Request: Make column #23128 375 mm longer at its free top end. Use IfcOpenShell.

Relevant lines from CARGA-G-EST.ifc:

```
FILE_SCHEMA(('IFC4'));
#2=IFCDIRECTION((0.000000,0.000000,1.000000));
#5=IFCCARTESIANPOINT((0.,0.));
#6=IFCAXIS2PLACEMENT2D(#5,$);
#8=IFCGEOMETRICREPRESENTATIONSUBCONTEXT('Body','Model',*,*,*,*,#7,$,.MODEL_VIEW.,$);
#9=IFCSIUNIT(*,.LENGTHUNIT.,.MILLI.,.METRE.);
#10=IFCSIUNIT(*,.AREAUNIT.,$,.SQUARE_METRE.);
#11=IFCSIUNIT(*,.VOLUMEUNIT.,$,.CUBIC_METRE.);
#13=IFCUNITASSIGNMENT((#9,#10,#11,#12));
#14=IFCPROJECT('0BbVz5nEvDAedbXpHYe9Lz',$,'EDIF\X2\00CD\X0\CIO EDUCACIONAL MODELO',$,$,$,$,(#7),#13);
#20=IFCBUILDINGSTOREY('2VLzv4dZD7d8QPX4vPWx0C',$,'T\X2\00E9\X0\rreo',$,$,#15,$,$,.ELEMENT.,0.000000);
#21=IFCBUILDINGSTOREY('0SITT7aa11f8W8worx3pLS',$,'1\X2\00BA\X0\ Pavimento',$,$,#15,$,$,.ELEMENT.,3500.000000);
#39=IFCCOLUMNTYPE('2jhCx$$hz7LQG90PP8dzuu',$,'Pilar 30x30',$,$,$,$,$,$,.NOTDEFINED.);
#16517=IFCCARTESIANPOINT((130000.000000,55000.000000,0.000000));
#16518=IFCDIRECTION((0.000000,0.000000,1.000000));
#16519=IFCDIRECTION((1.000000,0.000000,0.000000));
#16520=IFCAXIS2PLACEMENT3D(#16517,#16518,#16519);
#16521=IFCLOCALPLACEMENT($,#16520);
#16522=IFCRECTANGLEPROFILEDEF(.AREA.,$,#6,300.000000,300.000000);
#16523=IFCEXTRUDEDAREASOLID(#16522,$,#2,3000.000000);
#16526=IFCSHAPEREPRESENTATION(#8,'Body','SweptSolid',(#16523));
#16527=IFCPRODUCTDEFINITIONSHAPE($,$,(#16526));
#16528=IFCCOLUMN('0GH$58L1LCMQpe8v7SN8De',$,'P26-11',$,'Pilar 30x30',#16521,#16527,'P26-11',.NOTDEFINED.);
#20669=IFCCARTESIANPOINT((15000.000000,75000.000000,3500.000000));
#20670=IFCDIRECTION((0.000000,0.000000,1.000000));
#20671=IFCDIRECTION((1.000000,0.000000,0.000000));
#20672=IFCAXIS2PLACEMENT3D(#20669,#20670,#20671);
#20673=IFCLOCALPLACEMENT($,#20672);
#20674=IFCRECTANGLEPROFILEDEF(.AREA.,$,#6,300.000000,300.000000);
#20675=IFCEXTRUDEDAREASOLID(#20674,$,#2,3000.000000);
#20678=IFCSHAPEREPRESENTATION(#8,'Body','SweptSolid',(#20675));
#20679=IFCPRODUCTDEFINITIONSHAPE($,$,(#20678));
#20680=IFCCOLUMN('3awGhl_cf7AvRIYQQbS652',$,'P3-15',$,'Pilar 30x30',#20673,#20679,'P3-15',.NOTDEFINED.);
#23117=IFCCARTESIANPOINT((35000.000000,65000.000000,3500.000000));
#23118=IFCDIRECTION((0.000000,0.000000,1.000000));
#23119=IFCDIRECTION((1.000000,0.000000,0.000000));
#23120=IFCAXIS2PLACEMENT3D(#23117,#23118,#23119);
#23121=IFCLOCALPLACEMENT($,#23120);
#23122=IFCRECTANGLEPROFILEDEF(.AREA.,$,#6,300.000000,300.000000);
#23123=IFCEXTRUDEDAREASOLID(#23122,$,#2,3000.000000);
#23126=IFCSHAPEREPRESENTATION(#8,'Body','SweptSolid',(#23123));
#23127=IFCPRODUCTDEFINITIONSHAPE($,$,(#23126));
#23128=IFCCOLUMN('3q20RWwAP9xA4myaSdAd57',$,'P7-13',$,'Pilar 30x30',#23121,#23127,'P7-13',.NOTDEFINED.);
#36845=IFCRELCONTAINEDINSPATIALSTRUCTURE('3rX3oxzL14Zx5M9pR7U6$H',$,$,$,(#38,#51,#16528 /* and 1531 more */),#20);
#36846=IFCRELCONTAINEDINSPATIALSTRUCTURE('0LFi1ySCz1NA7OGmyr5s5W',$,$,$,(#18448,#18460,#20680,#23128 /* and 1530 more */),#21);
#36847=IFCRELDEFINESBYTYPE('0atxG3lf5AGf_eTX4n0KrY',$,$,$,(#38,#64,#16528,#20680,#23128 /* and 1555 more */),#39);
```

```python
import ifcopenshell
import ifcopenshell.util.representation

model = ifcopenshell.open("CARGA-G-EST.ifc")

member = model.by_guid("3q20RWwAP9xA4myaSdAd57")
change = 375.0

# The extrusion runs towards the end named, so only its depth changes.
body = ifcopenshell.util.representation.get_representation(member, "Model", "Body")
solid = body.Items[0]
old_length = solid.Depth
solid.Depth += change

print(f"length {old_length:g} -> {solid.Depth:g}")

model.write("CARGA-G-EST-out.ifc")
```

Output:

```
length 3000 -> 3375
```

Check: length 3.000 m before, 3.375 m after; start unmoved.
